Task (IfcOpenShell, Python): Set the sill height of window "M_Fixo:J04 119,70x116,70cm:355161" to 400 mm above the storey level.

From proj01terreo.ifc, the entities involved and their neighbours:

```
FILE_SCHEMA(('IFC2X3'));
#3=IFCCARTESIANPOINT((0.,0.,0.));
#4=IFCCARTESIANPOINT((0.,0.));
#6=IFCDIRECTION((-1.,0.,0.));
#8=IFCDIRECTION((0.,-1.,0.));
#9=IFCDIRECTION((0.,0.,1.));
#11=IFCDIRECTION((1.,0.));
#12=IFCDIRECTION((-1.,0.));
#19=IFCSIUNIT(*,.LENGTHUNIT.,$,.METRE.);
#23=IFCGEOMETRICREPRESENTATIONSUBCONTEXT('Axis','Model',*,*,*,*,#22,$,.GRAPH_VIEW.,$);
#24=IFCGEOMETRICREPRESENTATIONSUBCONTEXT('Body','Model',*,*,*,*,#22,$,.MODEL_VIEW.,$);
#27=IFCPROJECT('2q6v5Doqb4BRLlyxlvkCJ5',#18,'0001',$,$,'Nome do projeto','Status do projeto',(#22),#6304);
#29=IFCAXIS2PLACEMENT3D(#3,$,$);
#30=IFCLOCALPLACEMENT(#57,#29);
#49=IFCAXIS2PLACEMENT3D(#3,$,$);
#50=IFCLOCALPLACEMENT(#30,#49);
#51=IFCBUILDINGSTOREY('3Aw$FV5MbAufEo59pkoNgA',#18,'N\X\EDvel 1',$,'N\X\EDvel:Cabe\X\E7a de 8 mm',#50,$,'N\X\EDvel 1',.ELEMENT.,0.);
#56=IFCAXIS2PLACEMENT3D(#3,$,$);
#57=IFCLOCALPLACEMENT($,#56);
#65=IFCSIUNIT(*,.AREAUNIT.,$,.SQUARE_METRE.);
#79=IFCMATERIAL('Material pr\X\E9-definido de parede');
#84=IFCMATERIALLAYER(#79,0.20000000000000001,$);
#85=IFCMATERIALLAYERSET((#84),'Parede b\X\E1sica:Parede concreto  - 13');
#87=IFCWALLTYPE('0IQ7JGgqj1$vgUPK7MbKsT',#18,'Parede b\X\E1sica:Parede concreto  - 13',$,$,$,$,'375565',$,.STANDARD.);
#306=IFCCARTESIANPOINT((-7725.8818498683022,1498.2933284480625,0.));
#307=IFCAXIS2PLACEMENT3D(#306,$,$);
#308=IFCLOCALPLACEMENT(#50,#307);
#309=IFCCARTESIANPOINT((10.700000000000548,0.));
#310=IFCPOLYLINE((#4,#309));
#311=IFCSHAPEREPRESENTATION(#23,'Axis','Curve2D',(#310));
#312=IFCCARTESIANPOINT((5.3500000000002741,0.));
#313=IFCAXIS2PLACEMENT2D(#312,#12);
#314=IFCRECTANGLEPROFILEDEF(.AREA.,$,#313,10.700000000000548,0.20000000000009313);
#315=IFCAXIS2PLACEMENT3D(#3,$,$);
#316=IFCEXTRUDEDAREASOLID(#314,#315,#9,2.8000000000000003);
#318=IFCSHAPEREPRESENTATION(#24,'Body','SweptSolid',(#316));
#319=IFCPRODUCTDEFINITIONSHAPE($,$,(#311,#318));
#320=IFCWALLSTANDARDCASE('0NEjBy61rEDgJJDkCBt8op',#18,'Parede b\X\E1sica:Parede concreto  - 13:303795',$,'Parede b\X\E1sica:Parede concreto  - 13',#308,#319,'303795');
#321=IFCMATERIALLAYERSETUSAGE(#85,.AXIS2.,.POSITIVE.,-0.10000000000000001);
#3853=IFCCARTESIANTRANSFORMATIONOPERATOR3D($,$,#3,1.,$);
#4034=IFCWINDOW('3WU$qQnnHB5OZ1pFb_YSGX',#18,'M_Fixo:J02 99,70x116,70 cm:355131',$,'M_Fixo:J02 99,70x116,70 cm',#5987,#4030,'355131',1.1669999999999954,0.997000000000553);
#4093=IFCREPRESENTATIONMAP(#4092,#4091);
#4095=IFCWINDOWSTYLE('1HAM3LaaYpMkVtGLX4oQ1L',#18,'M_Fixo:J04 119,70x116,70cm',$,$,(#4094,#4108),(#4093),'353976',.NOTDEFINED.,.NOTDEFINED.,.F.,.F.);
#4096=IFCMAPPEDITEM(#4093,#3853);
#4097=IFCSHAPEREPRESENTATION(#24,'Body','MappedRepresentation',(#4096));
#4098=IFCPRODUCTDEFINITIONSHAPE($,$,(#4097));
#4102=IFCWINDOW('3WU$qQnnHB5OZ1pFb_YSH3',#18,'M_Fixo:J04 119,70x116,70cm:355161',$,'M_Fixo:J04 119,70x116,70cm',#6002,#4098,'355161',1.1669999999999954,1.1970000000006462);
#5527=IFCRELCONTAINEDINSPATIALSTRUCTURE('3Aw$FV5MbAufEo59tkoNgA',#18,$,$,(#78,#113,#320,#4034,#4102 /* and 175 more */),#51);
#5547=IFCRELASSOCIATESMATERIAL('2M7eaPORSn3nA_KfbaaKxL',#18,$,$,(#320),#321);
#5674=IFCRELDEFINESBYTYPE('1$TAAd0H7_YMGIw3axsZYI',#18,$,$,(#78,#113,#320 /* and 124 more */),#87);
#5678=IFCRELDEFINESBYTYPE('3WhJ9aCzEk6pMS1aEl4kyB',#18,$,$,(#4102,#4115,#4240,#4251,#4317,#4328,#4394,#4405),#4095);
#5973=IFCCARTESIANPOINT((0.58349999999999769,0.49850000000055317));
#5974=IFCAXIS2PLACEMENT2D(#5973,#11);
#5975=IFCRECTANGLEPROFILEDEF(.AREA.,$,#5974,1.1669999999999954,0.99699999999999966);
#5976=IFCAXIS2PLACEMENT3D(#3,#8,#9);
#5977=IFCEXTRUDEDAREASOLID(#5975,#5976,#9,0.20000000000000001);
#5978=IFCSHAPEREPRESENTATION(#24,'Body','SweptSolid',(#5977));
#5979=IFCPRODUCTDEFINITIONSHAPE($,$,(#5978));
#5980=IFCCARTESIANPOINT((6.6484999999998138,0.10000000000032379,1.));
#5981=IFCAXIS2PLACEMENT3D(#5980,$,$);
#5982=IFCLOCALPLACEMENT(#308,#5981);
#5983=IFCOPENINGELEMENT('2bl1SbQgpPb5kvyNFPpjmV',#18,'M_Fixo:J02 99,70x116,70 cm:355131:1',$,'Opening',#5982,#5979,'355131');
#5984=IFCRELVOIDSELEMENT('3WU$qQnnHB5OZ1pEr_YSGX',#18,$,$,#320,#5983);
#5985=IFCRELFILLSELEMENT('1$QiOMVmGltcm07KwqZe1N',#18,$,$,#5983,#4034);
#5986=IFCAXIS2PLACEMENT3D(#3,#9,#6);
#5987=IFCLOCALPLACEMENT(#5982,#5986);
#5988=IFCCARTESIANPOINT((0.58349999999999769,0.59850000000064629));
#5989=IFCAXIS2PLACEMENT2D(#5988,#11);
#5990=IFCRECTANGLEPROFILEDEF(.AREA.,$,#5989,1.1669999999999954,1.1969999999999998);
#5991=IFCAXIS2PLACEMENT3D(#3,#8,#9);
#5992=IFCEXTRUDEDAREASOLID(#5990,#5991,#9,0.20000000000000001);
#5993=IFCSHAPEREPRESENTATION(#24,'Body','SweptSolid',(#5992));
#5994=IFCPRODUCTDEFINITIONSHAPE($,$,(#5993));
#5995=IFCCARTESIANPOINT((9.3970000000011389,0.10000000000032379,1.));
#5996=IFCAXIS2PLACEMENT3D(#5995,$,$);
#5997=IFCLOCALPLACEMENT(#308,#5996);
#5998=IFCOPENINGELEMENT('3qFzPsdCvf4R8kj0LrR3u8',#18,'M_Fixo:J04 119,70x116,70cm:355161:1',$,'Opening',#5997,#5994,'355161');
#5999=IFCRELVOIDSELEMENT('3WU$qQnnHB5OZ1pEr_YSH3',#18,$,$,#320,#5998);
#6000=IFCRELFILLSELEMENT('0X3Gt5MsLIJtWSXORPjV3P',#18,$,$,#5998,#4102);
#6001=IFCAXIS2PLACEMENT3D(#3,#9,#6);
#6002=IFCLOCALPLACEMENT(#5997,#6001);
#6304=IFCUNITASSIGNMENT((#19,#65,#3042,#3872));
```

```python
import numpy as np
import ifcopenshell
import ifcopenshell.api.geometry
import ifcopenshell.geom
import ifcopenshell.util.element
import ifcopenshell.util.placement
import ifcopenshell.util.shape
import ifcopenshell.util.unit

model = ifcopenshell.open("proj01terreo.ifc")
unit_scale = ifcopenshell.util.unit.calculate_unit_scale(model)

window = model.by_guid("3WU$qQnnHB5OZ1pFb_YSH3")
opening = window.FillsVoids[0].RelatingOpeningElement
storey = ifcopenshell.util.element.get_container(window, ifc_class="IfcBuildingStorey")
level = ifcopenshell.util.placement.get_local_placement(storey.ObjectPlacement)[2, 3]

# The opening's origin need not be at the sill, so measure its lowest point.
shape = ifcopenshell.geom.create_shape(ifcopenshell.geom.settings(), opening)
bottom = ifcopenshell.util.shape.get_shape_bottom_elevation(shape, shape.geometry) / unit_scale
dz = level + 0.4 / unit_scale - bottom

shift = np.array([0.0, 0.0, dz])
# The window is placed relative to its opening, so it follows when the opening moves.
matrix = ifcopenshell.util.placement.get_local_placement(opening.ObjectPlacement)
matrix[:3, 3] += shift
ifcopenshell.api.geometry.edit_object_placement(
    model, product=opening, matrix=matrix, is_si=False, should_transform_children=True
)

print(f"moved by {dz * unit_scale:+.3f} m")

model.write("proj01terreo_v2.ifc")
```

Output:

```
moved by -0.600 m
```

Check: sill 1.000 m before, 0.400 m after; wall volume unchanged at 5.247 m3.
